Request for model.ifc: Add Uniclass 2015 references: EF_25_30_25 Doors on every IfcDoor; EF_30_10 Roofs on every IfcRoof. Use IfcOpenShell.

First a look at what the model holds.

```python
import ifcopenshell

model = ifcopenshell.open("model.ifc")
print(model.schema)
print("classifications:", [c.Name for c in model.by_type("IfcClassification")])
for ifc_class in ("IfcDoor", "IfcRoof", "IfcStair", "IfcWall", "IfcWindow"):
    print(ifc_class, len(model.by_type(ifc_class)))
```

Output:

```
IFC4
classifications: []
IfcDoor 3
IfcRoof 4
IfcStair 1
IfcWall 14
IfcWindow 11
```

```python
import ifcopenshell
import ifcopenshell.api.classification

model = ifcopenshell.open("model.ifc")

system = ifcopenshell.api.classification.add_classification(model, classification="Uniclass 2015")

codes = {
    "IfcDoor": ("EF_25_30_25", "Doors"),
    "IfcRoof": ("EF_30_10", "Roofs"),
}
for ifc_class, (code, name) in codes.items():
    products = model.by_type(ifc_class)
    ifcopenshell.api.classification.add_reference(
        model, products=products, classification=system, identification=code, name=name
    )
    print(code, len(products))

model.write("model_rev.ifc")
```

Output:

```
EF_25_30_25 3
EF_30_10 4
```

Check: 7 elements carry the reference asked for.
